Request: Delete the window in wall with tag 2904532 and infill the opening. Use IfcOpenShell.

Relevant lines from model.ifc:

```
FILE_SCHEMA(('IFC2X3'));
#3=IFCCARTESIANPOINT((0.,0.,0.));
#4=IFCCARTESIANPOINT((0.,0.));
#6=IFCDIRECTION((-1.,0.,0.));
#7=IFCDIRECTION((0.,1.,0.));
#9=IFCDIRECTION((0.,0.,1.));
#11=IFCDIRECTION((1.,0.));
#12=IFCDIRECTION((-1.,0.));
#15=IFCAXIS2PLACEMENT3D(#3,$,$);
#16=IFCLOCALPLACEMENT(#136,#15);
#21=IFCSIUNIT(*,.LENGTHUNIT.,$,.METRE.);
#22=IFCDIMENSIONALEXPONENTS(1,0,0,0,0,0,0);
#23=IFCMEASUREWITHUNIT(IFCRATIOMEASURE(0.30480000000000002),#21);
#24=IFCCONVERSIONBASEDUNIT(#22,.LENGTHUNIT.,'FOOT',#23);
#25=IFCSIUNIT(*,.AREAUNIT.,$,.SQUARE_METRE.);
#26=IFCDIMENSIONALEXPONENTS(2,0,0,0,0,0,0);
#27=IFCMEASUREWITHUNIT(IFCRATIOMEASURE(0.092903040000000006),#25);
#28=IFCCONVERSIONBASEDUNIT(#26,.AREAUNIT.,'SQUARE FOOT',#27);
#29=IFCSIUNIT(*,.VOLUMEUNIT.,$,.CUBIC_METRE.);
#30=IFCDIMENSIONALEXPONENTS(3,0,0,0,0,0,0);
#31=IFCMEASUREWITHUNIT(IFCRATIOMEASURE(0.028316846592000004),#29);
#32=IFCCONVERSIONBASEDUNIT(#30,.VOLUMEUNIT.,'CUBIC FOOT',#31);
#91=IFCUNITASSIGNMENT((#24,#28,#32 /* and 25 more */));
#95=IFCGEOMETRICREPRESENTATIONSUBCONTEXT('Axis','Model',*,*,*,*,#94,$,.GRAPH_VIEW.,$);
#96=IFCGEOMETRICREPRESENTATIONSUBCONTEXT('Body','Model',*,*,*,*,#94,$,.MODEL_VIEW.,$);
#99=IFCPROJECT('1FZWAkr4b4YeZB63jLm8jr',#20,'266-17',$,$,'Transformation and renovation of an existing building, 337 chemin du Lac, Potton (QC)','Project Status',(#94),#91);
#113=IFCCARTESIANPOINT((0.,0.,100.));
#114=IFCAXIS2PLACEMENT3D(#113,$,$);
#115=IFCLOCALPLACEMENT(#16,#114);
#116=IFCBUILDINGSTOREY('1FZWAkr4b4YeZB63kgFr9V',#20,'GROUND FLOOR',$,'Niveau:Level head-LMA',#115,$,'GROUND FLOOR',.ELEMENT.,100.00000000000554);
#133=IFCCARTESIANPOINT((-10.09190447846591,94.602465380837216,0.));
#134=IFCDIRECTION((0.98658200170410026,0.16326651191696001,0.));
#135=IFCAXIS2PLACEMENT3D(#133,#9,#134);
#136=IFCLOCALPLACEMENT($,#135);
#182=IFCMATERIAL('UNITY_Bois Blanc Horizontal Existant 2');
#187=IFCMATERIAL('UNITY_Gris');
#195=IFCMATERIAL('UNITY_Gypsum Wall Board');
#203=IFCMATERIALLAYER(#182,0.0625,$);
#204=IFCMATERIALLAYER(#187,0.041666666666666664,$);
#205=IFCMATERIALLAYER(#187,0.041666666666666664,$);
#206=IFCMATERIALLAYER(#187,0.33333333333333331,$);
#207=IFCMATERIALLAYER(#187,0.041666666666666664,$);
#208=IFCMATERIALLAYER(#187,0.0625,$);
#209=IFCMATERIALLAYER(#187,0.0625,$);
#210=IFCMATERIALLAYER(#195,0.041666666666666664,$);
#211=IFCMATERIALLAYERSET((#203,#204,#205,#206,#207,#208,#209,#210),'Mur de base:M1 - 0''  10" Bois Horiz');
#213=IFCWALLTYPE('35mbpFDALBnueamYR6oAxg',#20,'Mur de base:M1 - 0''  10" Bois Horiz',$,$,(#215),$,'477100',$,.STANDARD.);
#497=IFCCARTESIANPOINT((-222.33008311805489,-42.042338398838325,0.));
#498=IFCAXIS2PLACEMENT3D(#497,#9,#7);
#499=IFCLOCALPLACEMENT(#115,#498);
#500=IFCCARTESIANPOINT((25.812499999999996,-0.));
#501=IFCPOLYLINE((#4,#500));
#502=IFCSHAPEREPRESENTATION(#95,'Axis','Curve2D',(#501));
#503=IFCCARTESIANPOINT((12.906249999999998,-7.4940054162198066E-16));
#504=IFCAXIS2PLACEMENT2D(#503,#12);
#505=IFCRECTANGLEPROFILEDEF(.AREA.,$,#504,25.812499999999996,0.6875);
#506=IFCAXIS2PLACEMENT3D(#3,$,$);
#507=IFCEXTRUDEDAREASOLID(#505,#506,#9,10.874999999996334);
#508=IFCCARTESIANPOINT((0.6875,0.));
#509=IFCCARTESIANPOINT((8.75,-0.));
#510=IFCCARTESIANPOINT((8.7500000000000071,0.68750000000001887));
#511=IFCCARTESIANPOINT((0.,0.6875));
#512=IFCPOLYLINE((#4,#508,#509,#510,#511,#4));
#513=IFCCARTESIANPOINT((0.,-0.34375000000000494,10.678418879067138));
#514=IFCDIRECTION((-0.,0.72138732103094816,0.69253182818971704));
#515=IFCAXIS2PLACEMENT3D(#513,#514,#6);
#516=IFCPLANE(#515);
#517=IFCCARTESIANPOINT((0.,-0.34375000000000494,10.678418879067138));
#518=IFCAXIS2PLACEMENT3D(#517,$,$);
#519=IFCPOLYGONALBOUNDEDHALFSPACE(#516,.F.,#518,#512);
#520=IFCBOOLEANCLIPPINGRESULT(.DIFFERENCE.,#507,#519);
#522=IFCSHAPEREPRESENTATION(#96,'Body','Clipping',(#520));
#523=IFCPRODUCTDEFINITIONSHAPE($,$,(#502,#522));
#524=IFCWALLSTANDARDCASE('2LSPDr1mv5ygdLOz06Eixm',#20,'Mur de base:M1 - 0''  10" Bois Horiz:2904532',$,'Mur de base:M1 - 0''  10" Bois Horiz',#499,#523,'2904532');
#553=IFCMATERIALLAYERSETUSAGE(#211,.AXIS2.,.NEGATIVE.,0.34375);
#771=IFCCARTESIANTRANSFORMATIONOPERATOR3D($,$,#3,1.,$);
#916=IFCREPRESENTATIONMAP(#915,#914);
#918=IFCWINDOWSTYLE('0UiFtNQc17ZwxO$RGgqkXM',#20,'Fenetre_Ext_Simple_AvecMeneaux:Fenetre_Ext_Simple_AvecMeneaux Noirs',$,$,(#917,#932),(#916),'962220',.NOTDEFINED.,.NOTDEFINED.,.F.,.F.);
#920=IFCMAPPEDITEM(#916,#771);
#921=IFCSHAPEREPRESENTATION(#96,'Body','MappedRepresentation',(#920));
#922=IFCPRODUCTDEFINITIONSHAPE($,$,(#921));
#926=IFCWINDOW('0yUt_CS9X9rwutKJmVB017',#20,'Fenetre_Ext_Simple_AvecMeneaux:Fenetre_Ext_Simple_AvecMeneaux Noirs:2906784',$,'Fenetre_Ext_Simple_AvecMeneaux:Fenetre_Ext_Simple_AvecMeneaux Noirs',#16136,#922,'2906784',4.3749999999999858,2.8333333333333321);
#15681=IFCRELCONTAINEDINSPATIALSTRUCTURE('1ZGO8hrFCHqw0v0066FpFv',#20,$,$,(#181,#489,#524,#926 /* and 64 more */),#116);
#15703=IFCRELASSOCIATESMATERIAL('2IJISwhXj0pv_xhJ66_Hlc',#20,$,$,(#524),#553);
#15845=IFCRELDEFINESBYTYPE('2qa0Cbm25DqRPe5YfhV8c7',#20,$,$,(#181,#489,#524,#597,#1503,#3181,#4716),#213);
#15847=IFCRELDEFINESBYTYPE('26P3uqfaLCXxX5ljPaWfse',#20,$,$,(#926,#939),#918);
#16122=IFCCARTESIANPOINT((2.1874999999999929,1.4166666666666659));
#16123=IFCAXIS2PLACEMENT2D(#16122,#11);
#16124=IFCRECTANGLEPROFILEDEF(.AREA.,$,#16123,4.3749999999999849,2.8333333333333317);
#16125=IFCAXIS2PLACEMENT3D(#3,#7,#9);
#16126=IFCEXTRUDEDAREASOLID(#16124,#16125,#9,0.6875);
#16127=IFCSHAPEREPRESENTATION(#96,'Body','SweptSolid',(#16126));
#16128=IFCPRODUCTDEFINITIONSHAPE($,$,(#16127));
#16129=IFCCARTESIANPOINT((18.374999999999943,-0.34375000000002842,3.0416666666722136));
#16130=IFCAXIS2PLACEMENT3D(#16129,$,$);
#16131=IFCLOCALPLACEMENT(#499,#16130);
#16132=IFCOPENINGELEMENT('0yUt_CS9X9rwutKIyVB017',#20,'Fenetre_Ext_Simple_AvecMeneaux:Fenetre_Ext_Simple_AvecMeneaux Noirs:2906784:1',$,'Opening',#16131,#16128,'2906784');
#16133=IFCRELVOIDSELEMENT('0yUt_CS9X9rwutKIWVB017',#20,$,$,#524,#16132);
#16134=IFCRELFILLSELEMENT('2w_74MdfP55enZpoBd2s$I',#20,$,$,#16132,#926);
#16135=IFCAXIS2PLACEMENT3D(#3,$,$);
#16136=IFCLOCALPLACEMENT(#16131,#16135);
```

```python
import ifcopenshell
import ifcopenshell.api.feature
import ifcopenshell.api.root
import ifcopenshell.geom
import ifcopenshell.util.shape

model = ifcopenshell.open("model.ifc")
settings = ifcopenshell.geom.settings()


def volume(element):
    """Net volume in cubic metres, openings subtracted."""
    shape = ifcopenshell.geom.create_shape(settings, element)
    return ifcopenshell.util.shape.get_volume(shape.geometry)


window = model.by_guid("0yUt_CS9X9rwutKJmVB017")
opening = window.FillsVoids[0].RelatingOpeningElement
wall = opening.VoidsElements[0].RelatingBuildingElement
before = volume(wall)

ifcopenshell.api.root.remove_product(model, product=window)
ifcopenshell.api.feature.remove_feature(model, feature=opening)

after = volume(wall)

print(f"wall volume {before:.3f} -> {after:.3f} m3")

model.write("model_updated.ifc")
```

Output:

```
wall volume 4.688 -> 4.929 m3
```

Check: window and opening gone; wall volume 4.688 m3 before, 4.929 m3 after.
